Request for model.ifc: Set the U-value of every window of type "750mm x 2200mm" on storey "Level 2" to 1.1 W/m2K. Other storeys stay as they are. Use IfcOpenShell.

First a look at what the model holds.

```python
import ifcopenshell
import ifcopenshell.util.element

model = ifcopenshell.open("model.ifc")
print(model.schema)
storey = next(s for s in model.by_type("IfcBuildingStorey") if s.Name == "Level 2")
windows = [e for e in ifcopenshell.util.element.get_decomposition(storey) if e.is_a("IfcWindow")]
seen = {}
for e in windows:
    element_type = ifcopenshell.util.element.get_type(e)
    key = (element_type.Name if element_type != e and element_type else None, ifcopenshell.util.element.get_pset(e, "Pset_WindowCommon", "ThermalTransmittance"))
    seen[key] = seen.get(key, 0) + 1
for (name, value), count in sorted(seen.items(), key=str):
    print(count, "x", name, "|", value)
```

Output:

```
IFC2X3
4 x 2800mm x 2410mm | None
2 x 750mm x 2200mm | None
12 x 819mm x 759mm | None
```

```python
import ifcopenshell
import ifcopenshell.api.pset
import ifcopenshell.util.element

model = ifcopenshell.open("model.ifc")

storey = next(s for s in model.by_type("IfcBuildingStorey") if s.Name == "Level 2")
windows = [e for e in ifcopenshell.util.element.get_decomposition(storey) if e.is_a("IfcWindow")]

count = 0
for e in windows:
    element_type = ifcopenshell.util.element.get_type(e)
    if element_type in (None, e) or element_type.Name != "750mm x 2200mm":
        continue
    # add_pset returns the element's existing set when there is one.
    pset = ifcopenshell.api.pset.add_pset(model, product=e, name="Pset_WindowCommon")
    ifcopenshell.api.pset.edit_pset(model, pset=pset, properties={"ThermalTransmittance": 1.1})
    count += 1

print(count, "windows updated")

model.write("model_v2.ifc")
```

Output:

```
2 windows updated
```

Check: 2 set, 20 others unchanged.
